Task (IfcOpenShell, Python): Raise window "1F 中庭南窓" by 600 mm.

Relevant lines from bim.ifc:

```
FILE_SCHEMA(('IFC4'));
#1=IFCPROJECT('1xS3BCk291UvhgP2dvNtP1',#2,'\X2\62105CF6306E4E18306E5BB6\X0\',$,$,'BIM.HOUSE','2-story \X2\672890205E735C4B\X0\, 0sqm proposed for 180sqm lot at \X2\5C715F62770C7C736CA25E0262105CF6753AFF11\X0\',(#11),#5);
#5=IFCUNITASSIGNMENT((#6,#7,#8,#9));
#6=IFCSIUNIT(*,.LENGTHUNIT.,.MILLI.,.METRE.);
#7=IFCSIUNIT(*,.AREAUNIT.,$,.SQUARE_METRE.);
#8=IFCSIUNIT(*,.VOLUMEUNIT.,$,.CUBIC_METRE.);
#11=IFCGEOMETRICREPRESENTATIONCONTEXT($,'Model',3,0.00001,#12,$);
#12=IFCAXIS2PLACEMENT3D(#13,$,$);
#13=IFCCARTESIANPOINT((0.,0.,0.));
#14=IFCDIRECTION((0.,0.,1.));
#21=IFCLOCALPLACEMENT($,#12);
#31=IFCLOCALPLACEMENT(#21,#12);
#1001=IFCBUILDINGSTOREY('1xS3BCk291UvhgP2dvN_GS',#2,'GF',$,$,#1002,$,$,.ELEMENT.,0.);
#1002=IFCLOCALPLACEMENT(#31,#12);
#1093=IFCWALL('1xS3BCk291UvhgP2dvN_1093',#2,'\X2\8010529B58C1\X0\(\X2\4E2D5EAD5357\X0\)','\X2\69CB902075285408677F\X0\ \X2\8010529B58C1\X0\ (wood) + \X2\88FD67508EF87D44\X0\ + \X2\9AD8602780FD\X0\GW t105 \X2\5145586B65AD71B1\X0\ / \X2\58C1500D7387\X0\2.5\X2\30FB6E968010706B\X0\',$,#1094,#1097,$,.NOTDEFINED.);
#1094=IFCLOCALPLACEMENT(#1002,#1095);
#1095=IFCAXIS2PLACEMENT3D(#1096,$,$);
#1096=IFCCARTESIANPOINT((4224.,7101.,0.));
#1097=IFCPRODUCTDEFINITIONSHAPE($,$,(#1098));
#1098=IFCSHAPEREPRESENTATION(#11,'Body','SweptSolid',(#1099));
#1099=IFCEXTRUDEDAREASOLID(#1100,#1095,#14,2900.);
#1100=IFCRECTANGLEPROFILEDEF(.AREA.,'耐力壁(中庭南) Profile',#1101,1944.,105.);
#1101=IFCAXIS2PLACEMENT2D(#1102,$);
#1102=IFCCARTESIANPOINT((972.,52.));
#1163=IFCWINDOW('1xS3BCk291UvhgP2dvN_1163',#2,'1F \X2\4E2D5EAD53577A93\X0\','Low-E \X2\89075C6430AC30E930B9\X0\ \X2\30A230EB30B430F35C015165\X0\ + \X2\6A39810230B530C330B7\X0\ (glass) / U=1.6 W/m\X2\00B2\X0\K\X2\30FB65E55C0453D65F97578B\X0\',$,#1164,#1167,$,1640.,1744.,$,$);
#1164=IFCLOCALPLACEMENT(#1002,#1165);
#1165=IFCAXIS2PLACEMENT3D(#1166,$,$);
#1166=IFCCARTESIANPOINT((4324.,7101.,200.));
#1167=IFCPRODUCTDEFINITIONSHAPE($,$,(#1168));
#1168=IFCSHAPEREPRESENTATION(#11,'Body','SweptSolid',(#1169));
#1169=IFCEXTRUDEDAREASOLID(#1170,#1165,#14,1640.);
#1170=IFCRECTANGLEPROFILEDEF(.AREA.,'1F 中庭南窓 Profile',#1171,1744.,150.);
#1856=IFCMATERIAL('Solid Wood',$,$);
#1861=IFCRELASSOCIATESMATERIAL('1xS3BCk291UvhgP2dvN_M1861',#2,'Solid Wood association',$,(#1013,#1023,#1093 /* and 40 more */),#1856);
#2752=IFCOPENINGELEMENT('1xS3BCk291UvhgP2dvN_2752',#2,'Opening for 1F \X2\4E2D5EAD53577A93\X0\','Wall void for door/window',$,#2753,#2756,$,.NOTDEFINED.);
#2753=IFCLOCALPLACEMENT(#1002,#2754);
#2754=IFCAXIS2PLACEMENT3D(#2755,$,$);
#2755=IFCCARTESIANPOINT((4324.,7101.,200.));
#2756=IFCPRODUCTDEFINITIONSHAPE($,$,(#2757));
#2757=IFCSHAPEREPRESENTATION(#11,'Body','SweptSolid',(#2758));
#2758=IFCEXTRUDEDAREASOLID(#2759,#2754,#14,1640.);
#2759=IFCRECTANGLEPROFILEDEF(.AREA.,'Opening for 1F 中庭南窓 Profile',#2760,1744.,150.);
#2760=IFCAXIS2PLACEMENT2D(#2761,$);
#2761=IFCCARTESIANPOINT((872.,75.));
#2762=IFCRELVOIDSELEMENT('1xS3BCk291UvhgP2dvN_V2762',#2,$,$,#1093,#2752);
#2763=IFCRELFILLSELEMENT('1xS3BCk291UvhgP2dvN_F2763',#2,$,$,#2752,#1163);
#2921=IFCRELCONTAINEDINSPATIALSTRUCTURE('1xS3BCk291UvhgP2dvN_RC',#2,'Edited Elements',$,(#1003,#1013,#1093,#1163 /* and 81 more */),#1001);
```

```python
import numpy as np
import ifcopenshell
import ifcopenshell.api.geometry
import ifcopenshell.util.placement
import ifcopenshell.util.unit

model = ifcopenshell.open("bim.ifc")
unit_scale = ifcopenshell.util.unit.calculate_unit_scale(model)

window = model.by_guid("1xS3BCk291UvhgP2dvN_1163")
opening = window.FillsVoids[0].RelatingOpeningElement
dz = 600.0

shift = np.array([0.0, 0.0, dz])
# The window is not placed relative to its opening, so move both.
for product in (opening, window):
    matrix = ifcopenshell.util.placement.get_local_placement(product.ObjectPlacement)
    matrix[:3, 3] += shift
    ifcopenshell.api.geometry.edit_object_placement(model, product=product, matrix=matrix, is_si=False)

print(f"moved by {dz * unit_scale:+.3f} m")

model.write("bim_updated.ifc")
```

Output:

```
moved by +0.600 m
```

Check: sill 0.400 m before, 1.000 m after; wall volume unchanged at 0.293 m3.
